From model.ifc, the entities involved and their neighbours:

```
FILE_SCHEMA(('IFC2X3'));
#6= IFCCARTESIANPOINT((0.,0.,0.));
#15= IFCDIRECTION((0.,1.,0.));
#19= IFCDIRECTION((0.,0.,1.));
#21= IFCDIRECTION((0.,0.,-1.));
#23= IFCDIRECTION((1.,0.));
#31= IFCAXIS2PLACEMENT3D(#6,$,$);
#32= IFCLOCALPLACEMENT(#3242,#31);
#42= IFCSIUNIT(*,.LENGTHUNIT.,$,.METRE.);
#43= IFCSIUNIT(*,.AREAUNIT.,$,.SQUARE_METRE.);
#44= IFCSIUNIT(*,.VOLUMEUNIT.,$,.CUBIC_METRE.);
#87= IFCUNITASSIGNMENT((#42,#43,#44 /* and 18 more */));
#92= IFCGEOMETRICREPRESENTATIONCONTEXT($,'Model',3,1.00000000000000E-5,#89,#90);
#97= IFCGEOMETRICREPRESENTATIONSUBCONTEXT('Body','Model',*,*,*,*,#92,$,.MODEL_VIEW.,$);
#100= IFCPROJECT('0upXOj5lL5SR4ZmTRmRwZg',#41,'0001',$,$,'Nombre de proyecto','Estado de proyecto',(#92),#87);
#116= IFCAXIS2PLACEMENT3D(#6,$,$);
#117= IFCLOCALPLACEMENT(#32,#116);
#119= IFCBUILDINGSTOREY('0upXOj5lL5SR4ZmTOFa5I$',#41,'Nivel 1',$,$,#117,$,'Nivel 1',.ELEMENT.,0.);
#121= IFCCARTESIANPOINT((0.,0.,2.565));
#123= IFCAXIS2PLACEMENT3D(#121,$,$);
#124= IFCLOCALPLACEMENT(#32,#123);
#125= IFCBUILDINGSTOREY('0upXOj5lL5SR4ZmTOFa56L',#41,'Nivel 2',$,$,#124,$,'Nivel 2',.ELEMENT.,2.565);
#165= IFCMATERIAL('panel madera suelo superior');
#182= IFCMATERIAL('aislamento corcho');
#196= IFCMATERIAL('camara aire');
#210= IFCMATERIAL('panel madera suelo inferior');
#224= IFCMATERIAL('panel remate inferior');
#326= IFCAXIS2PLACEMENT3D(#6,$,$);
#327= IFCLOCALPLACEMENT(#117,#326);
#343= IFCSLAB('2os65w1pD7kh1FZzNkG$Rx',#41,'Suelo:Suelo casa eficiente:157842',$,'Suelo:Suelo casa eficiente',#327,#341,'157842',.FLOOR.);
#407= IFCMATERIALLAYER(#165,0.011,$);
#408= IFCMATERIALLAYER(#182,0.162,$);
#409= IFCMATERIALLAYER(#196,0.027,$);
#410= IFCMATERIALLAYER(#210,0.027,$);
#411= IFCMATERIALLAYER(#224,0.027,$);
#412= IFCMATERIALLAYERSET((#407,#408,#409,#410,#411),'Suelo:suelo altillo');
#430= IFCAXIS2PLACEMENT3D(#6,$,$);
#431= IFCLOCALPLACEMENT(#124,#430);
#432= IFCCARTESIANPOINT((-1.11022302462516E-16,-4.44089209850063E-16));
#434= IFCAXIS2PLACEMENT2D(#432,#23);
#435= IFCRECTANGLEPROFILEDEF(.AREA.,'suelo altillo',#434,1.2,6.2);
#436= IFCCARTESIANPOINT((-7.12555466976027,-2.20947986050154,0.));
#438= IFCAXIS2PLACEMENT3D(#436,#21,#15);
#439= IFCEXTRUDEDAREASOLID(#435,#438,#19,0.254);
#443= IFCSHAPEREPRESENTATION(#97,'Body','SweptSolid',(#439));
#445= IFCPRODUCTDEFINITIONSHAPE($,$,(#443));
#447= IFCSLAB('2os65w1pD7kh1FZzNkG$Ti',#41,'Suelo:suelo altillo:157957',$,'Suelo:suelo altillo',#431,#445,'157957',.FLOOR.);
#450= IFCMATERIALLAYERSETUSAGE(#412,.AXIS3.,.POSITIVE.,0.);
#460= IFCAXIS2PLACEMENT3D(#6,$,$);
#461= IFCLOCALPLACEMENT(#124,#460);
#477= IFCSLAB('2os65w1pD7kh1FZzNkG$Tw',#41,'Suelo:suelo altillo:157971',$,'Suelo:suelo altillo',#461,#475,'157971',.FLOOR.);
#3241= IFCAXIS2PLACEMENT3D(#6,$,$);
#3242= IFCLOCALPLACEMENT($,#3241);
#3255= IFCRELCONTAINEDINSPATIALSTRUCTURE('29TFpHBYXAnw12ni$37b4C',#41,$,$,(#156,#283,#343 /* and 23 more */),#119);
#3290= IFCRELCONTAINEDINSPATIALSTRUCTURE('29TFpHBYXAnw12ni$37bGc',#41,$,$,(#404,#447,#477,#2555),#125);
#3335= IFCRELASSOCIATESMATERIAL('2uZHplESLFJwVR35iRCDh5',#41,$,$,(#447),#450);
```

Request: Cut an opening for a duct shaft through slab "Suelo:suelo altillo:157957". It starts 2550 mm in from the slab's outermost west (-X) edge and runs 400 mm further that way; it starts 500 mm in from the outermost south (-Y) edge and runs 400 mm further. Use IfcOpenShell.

```python
import numpy as np
import ifcopenshell
import ifcopenshell.api.feature
import ifcopenshell.api.geometry
import ifcopenshell.api.root
import ifcopenshell.geom
import ifcopenshell.util.placement
import ifcopenshell.util.representation
import ifcopenshell.util.shape
import ifcopenshell.util.unit

model = ifcopenshell.open("model.ifc")
unit_scale = ifcopenshell.util.unit.calculate_unit_scale(model)
settings = ifcopenshell.geom.settings()


def volume(element):
    """Net volume in cubic metres, openings subtracted."""
    shape = ifcopenshell.geom.create_shape(settings, element)
    return ifcopenshell.util.shape.get_volume(shape.geometry)


slab = model.by_guid("2os65w1pD7kh1FZzNkG$Ti")
before = volume(slab)

# Extent in the slab's own axes, in metres. The edges named are its -X and -Y sides.
slab_shape = ifcopenshell.geom.create_shape(settings, slab)
vertices = ifcopenshell.util.shape.get_vertices(slab_shape.geometry)
x_min, y_min, bottom = vertices.min(axis=0)
top = vertices[:, 2].max()

opening = ifcopenshell.api.root.create_entity(model, ifc_class="IfcOpeningElement", name="Duct shaft opening")
context = ifcopenshell.util.representation.get_context(model, "Model", "Body", "MODEL_VIEW")
width, depth = 0.4, 0.4
outline = [(0.0, 0.0), (width, 0.0), (width, depth), (0.0, depth), (0.0, 0.0)]
# Overshoot both faces by 50 mm so the cut is clean.
shape = ifcopenshell.api.geometry.add_slab_representation(
    model, context=context, depth=top - bottom + 0.1, polyline=outline
)
ifcopenshell.api.geometry.assign_representation(model, product=opening, representation=shape)

matrix = ifcopenshell.util.placement.get_local_placement(slab.ObjectPlacement)
matrix[:, 3] = matrix @ np.append(np.array([x_min + 2.55, y_min + 0.5, bottom - 0.05]) / unit_scale, 1.0)
ifcopenshell.api.geometry.edit_object_placement(model, product=opening, matrix=matrix, is_si=False)
ifcopenshell.api.feature.add_feature(model, feature=opening, element=slab)

after = volume(slab)

print(f"slab volume {before:.3f} -> {after:.3f} m3")

model.write("model_updated.ifc")
```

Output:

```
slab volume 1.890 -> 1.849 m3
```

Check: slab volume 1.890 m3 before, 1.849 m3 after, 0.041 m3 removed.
